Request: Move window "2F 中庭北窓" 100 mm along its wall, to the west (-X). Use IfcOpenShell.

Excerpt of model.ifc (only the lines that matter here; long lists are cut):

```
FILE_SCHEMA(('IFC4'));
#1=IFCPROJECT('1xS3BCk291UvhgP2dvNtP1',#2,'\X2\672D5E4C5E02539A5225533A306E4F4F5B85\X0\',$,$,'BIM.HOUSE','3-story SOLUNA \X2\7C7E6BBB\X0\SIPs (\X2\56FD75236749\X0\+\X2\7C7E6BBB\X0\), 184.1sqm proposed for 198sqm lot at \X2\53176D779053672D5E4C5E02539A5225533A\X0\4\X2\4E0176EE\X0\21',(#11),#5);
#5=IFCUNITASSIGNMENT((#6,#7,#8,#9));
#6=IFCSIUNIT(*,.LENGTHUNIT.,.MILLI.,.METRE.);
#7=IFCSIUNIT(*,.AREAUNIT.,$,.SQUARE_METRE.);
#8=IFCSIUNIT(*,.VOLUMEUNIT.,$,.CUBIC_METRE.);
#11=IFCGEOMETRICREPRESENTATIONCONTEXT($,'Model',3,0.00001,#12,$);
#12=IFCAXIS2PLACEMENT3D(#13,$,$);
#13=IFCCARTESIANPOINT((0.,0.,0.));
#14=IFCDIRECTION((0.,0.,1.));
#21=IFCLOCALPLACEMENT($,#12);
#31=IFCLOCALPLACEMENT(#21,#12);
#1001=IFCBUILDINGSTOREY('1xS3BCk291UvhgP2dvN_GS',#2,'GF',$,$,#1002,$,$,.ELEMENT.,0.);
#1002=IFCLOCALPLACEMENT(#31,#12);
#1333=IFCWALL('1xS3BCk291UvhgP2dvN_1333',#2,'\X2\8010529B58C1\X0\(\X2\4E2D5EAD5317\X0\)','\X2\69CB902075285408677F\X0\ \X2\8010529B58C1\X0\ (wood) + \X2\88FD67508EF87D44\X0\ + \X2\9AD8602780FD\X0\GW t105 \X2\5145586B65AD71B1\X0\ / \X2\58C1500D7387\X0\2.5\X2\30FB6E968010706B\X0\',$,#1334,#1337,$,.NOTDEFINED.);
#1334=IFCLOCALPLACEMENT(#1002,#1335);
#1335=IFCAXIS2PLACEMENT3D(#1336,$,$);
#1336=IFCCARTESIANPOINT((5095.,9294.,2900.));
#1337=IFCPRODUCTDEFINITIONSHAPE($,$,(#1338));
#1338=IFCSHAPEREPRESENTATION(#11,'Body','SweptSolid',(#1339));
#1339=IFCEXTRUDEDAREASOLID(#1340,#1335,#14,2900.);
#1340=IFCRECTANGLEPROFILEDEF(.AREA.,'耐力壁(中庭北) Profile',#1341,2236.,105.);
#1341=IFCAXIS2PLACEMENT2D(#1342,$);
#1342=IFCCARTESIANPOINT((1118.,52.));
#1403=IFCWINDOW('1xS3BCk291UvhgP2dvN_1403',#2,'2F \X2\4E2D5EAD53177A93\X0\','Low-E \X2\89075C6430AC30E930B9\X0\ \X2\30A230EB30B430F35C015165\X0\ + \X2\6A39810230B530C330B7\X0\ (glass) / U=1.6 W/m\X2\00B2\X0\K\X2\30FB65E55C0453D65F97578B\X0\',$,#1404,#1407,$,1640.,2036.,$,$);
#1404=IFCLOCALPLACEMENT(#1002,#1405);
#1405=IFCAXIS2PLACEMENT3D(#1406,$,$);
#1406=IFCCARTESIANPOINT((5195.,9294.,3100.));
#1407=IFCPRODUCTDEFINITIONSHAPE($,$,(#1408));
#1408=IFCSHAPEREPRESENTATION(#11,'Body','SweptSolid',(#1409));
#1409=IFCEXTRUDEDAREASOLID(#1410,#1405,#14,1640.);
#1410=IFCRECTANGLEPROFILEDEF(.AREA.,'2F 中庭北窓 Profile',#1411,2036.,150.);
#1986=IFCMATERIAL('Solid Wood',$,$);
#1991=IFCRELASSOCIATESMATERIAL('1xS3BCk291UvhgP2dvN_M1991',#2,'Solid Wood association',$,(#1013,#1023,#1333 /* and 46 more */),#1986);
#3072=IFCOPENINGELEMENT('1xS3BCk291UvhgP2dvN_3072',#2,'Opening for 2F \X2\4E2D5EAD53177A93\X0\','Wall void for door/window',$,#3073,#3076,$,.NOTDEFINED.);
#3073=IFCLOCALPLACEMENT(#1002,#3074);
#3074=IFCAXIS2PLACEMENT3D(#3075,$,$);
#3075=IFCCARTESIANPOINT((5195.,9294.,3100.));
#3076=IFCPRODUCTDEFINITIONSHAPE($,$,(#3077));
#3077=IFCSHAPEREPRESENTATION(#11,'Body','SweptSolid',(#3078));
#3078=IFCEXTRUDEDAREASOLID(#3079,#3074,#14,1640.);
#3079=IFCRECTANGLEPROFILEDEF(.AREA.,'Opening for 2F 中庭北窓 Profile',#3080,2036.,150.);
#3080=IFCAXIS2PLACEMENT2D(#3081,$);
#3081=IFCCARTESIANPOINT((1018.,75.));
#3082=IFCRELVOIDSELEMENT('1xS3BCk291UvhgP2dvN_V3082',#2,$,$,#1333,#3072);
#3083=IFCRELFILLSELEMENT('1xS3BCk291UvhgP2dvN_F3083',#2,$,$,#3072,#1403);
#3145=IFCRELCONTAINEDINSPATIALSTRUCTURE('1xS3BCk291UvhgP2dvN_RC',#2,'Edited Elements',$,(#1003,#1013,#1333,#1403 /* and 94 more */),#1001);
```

```python
import ifcopenshell
import ifcopenshell.api.geometry
import ifcopenshell.util.placement
import ifcopenshell.util.unit

model = ifcopenshell.open("model.ifc")
unit_scale = ifcopenshell.util.unit.calculate_unit_scale(model)

window = model.by_id(1403)
opening = window.FillsVoids[0].RelatingOpeningElement
wall = opening.VoidsElements[0].RelatingBuildingElement

wall_matrix = ifcopenshell.util.placement.get_local_placement(wall.ObjectPlacement)
shift = wall_matrix[:3, 0] * -0.1 / unit_scale
before = ifcopenshell.util.placement.get_local_placement(window.ObjectPlacement)[:3, 3].copy()

# The window is not placed relative to its opening, so move both.
for product in (opening, window):
    matrix = ifcopenshell.util.placement.get_local_placement(product.ObjectPlacement)
    matrix[:3, 3] += shift
    ifcopenshell.api.geometry.edit_object_placement(model, product=product, matrix=matrix, is_si=False)

after = ifcopenshell.util.placement.get_local_placement(window.ObjectPlacement)[:3, 3]
print("window moved by", (after - before).round(3) + 0.0)

model.write("model_rev.ifc")
```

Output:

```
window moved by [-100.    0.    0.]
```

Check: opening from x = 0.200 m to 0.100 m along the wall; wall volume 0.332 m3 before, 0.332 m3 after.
